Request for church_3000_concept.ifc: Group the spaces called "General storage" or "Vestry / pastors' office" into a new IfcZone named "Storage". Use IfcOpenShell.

First a look at what the model holds.

```python
import ifcopenshell

model = ifcopenshell.open("church_3000_concept.ifc")
print(model.schema)
seen = {}
for space in model.by_type("IfcSpace"):
    seen[space.LongName] = seen.get(space.LongName, 0) + 1
for name, count in sorted(seen.items(), key=str):
    print(count, "x", name)
print("zones:", [z.Name for z in model.by_type("IfcZone")][:20])
```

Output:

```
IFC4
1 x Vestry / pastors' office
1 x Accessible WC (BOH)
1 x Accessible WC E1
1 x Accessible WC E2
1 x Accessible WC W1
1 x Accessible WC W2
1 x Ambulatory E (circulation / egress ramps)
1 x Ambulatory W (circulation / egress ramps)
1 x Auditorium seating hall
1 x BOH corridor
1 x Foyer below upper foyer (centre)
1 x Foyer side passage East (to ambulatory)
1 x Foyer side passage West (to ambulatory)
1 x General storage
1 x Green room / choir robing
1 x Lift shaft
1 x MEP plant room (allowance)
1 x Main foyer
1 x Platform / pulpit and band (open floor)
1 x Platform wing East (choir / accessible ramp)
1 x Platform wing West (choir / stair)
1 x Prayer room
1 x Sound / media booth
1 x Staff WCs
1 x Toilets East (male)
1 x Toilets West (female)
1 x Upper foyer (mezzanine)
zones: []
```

```python
import ifcopenshell
import ifcopenshell.api.group
import ifcopenshell.api.root

model = ifcopenshell.open("church_3000_concept.ifc")

names = {"General storage", "Vestry / pastors' office"}
spaces = [s for s in model.by_type("IfcSpace") if s.LongName in names]

zone = ifcopenshell.api.root.create_entity(model, ifc_class="IfcZone", name="Storage")
ifcopenshell.api.group.assign_group(model, products=spaces, group=zone)
print(len(spaces), "spaces in", zone.Name)

model.write("church_3000_concept_edited.ifc")
```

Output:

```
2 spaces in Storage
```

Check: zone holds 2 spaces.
